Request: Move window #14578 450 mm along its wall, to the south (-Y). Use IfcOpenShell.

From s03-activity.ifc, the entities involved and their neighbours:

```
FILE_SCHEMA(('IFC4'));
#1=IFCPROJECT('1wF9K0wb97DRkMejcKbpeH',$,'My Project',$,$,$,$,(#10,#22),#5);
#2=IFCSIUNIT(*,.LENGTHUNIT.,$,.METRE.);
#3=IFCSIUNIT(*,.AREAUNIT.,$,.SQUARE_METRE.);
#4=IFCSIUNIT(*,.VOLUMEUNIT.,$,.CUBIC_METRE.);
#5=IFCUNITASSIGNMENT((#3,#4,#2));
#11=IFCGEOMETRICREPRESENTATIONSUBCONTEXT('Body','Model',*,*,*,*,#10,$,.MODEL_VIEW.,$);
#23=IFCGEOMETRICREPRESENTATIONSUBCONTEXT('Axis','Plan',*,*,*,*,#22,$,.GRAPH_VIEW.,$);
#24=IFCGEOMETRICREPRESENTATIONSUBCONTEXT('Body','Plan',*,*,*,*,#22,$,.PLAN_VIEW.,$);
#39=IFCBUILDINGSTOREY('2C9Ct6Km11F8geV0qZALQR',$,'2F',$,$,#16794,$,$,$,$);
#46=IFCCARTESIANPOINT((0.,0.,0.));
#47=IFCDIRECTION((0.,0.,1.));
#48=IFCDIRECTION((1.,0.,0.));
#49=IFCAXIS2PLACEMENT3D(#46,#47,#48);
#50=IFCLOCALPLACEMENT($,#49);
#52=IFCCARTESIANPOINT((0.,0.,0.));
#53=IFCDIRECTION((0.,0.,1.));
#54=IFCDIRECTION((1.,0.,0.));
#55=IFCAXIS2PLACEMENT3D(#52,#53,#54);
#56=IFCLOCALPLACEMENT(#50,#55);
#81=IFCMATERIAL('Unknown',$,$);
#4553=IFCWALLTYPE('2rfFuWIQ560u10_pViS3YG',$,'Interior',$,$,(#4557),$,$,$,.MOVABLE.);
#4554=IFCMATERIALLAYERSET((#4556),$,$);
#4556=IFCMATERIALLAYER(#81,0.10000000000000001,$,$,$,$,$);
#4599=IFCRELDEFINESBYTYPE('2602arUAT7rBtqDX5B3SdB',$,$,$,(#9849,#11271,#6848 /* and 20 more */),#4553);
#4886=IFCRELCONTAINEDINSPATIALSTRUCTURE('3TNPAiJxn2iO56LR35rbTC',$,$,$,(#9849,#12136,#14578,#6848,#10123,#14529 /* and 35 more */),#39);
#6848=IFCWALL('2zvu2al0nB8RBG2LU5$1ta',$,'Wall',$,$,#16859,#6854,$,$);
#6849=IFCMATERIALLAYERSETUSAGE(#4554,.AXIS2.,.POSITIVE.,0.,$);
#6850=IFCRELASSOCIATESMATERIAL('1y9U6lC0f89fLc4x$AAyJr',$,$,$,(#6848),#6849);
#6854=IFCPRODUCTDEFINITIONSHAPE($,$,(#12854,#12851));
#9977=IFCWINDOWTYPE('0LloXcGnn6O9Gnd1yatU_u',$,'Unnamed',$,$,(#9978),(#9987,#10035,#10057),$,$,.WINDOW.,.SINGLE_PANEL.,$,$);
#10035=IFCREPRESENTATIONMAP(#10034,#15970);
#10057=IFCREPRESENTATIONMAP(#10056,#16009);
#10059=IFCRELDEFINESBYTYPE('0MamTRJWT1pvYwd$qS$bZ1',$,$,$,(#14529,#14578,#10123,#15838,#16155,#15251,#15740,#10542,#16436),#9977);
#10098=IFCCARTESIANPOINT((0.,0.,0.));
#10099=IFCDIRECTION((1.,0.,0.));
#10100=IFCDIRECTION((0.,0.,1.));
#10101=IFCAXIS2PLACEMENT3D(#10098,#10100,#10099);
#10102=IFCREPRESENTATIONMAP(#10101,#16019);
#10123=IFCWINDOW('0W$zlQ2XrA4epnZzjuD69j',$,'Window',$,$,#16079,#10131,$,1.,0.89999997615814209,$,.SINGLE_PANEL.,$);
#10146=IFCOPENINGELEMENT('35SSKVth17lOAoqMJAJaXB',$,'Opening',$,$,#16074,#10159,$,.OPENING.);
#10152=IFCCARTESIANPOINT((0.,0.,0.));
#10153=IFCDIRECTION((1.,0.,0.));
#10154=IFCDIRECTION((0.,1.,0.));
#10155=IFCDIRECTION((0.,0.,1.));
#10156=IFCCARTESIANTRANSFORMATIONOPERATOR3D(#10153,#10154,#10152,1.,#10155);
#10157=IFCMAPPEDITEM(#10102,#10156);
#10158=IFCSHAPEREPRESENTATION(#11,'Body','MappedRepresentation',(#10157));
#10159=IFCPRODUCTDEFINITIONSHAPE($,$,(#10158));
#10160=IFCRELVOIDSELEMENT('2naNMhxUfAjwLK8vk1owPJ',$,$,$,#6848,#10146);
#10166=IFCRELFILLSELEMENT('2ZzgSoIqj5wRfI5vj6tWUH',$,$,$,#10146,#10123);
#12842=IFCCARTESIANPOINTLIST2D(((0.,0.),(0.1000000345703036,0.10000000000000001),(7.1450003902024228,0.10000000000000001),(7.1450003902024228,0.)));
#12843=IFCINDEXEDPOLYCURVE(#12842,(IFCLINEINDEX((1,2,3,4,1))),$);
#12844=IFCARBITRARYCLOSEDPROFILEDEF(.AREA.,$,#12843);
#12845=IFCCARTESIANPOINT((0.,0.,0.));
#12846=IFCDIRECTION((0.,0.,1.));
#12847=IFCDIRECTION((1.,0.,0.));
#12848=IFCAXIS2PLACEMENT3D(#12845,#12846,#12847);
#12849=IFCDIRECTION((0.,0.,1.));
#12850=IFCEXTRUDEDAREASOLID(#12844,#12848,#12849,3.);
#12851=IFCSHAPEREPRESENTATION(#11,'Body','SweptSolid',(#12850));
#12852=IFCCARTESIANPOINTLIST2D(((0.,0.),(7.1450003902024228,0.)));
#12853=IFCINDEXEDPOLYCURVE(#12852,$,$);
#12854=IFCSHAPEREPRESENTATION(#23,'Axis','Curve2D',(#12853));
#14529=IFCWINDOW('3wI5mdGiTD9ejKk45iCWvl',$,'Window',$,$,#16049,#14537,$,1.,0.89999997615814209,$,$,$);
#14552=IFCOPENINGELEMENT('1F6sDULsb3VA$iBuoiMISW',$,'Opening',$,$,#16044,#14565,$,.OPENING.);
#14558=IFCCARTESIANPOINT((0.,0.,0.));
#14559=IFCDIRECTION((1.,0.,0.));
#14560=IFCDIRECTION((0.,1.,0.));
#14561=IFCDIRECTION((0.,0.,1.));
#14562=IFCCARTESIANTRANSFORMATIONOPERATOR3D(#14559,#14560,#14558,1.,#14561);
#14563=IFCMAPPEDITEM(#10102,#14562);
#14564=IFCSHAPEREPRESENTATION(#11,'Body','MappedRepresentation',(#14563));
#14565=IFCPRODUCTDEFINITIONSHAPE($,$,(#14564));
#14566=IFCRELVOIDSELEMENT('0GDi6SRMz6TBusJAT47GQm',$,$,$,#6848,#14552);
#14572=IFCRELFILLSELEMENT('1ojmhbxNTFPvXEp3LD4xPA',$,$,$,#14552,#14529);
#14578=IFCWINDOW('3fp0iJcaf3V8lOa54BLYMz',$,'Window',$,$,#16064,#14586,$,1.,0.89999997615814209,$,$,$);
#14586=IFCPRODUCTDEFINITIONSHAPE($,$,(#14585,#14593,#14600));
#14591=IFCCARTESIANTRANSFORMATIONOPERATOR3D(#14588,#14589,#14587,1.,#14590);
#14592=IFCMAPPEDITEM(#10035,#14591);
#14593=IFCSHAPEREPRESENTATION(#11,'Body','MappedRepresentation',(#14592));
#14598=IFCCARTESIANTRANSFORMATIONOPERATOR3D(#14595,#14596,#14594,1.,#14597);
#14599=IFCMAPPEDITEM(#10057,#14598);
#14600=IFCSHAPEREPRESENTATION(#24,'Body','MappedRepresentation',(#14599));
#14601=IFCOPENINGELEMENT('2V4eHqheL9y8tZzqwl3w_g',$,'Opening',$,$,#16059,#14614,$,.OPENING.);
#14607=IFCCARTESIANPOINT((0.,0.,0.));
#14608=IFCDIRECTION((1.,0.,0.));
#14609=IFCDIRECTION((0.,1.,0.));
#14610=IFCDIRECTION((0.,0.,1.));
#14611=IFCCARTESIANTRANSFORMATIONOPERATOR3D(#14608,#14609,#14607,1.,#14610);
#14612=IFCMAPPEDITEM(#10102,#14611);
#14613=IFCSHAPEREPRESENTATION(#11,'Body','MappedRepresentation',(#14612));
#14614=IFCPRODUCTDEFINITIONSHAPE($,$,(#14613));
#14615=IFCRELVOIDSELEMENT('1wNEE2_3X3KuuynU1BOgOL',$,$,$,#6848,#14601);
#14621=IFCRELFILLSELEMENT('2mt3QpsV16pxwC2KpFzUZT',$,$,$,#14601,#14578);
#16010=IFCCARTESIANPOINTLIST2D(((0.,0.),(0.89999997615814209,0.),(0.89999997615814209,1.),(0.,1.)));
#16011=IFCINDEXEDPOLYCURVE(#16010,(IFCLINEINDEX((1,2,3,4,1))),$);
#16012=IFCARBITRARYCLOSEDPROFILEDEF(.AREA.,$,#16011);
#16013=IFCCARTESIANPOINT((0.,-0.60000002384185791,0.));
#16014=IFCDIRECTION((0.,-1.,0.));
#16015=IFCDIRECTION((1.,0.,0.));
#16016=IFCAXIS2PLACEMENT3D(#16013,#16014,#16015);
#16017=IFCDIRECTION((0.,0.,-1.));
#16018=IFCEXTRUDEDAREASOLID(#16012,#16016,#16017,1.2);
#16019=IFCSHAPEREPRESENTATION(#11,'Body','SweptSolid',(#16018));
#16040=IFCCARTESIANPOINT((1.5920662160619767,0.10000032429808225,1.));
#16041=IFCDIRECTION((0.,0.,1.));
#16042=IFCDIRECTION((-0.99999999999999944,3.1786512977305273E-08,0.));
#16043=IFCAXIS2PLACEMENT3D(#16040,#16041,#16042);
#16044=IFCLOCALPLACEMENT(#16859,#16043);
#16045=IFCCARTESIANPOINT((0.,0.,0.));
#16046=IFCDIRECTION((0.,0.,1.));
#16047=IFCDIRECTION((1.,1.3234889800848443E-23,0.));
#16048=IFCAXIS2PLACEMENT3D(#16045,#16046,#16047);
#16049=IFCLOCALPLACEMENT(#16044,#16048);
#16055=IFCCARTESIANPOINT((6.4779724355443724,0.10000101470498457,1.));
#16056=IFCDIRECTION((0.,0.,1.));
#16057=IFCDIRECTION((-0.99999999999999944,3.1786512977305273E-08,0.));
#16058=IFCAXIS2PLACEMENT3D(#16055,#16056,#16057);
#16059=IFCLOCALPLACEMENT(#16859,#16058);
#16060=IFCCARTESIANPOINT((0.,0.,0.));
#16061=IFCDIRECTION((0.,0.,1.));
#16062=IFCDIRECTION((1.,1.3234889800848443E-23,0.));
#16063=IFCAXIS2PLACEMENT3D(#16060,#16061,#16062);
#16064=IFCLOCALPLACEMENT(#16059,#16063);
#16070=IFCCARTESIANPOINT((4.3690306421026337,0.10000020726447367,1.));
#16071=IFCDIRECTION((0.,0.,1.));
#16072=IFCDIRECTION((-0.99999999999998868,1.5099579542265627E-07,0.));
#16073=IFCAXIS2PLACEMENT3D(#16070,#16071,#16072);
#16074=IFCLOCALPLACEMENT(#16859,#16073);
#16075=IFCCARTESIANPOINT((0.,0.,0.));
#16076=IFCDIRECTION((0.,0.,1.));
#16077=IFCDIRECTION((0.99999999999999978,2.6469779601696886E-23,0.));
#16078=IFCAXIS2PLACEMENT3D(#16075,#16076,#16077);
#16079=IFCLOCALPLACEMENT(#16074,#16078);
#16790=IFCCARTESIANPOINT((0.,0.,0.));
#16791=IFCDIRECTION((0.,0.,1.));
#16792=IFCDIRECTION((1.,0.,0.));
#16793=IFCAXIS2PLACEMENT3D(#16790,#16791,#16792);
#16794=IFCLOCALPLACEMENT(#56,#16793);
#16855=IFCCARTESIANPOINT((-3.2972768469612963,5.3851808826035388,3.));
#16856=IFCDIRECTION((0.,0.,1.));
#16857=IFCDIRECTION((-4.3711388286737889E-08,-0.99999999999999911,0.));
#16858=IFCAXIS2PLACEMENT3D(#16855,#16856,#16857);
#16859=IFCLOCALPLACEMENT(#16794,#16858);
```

```python
import ifcopenshell
import ifcopenshell.api.geometry
import ifcopenshell.util.placement

model = ifcopenshell.open("s03-activity.ifc")

window = model.by_guid("3fp0iJcaf3V8lOa54BLYMz")
opening = window.FillsVoids[0].RelatingOpeningElement
wall = opening.VoidsElements[0].RelatingBuildingElement

wall_matrix = ifcopenshell.util.placement.get_local_placement(wall.ObjectPlacement)
shift = wall_matrix[:3, 0] * 0.45
before = ifcopenshell.util.placement.get_local_placement(window.ObjectPlacement)[:3, 3].copy()

# The window is placed relative to its opening, so it follows when the opening moves.
matrix = ifcopenshell.util.placement.get_local_placement(opening.ObjectPlacement)
matrix[:3, 3] += shift
ifcopenshell.api.geometry.edit_object_placement(
    model, product=opening, matrix=matrix, is_si=False, should_transform_children=True
)

after = ifcopenshell.util.placement.get_local_placement(window.ObjectPlacement)[:3, 3]
print("window moved by", (after - before).round(3) + 0.0)

model.write("s03-activity_v2.ifc")
```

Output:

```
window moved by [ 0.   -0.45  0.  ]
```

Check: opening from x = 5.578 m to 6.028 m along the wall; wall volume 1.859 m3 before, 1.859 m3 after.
